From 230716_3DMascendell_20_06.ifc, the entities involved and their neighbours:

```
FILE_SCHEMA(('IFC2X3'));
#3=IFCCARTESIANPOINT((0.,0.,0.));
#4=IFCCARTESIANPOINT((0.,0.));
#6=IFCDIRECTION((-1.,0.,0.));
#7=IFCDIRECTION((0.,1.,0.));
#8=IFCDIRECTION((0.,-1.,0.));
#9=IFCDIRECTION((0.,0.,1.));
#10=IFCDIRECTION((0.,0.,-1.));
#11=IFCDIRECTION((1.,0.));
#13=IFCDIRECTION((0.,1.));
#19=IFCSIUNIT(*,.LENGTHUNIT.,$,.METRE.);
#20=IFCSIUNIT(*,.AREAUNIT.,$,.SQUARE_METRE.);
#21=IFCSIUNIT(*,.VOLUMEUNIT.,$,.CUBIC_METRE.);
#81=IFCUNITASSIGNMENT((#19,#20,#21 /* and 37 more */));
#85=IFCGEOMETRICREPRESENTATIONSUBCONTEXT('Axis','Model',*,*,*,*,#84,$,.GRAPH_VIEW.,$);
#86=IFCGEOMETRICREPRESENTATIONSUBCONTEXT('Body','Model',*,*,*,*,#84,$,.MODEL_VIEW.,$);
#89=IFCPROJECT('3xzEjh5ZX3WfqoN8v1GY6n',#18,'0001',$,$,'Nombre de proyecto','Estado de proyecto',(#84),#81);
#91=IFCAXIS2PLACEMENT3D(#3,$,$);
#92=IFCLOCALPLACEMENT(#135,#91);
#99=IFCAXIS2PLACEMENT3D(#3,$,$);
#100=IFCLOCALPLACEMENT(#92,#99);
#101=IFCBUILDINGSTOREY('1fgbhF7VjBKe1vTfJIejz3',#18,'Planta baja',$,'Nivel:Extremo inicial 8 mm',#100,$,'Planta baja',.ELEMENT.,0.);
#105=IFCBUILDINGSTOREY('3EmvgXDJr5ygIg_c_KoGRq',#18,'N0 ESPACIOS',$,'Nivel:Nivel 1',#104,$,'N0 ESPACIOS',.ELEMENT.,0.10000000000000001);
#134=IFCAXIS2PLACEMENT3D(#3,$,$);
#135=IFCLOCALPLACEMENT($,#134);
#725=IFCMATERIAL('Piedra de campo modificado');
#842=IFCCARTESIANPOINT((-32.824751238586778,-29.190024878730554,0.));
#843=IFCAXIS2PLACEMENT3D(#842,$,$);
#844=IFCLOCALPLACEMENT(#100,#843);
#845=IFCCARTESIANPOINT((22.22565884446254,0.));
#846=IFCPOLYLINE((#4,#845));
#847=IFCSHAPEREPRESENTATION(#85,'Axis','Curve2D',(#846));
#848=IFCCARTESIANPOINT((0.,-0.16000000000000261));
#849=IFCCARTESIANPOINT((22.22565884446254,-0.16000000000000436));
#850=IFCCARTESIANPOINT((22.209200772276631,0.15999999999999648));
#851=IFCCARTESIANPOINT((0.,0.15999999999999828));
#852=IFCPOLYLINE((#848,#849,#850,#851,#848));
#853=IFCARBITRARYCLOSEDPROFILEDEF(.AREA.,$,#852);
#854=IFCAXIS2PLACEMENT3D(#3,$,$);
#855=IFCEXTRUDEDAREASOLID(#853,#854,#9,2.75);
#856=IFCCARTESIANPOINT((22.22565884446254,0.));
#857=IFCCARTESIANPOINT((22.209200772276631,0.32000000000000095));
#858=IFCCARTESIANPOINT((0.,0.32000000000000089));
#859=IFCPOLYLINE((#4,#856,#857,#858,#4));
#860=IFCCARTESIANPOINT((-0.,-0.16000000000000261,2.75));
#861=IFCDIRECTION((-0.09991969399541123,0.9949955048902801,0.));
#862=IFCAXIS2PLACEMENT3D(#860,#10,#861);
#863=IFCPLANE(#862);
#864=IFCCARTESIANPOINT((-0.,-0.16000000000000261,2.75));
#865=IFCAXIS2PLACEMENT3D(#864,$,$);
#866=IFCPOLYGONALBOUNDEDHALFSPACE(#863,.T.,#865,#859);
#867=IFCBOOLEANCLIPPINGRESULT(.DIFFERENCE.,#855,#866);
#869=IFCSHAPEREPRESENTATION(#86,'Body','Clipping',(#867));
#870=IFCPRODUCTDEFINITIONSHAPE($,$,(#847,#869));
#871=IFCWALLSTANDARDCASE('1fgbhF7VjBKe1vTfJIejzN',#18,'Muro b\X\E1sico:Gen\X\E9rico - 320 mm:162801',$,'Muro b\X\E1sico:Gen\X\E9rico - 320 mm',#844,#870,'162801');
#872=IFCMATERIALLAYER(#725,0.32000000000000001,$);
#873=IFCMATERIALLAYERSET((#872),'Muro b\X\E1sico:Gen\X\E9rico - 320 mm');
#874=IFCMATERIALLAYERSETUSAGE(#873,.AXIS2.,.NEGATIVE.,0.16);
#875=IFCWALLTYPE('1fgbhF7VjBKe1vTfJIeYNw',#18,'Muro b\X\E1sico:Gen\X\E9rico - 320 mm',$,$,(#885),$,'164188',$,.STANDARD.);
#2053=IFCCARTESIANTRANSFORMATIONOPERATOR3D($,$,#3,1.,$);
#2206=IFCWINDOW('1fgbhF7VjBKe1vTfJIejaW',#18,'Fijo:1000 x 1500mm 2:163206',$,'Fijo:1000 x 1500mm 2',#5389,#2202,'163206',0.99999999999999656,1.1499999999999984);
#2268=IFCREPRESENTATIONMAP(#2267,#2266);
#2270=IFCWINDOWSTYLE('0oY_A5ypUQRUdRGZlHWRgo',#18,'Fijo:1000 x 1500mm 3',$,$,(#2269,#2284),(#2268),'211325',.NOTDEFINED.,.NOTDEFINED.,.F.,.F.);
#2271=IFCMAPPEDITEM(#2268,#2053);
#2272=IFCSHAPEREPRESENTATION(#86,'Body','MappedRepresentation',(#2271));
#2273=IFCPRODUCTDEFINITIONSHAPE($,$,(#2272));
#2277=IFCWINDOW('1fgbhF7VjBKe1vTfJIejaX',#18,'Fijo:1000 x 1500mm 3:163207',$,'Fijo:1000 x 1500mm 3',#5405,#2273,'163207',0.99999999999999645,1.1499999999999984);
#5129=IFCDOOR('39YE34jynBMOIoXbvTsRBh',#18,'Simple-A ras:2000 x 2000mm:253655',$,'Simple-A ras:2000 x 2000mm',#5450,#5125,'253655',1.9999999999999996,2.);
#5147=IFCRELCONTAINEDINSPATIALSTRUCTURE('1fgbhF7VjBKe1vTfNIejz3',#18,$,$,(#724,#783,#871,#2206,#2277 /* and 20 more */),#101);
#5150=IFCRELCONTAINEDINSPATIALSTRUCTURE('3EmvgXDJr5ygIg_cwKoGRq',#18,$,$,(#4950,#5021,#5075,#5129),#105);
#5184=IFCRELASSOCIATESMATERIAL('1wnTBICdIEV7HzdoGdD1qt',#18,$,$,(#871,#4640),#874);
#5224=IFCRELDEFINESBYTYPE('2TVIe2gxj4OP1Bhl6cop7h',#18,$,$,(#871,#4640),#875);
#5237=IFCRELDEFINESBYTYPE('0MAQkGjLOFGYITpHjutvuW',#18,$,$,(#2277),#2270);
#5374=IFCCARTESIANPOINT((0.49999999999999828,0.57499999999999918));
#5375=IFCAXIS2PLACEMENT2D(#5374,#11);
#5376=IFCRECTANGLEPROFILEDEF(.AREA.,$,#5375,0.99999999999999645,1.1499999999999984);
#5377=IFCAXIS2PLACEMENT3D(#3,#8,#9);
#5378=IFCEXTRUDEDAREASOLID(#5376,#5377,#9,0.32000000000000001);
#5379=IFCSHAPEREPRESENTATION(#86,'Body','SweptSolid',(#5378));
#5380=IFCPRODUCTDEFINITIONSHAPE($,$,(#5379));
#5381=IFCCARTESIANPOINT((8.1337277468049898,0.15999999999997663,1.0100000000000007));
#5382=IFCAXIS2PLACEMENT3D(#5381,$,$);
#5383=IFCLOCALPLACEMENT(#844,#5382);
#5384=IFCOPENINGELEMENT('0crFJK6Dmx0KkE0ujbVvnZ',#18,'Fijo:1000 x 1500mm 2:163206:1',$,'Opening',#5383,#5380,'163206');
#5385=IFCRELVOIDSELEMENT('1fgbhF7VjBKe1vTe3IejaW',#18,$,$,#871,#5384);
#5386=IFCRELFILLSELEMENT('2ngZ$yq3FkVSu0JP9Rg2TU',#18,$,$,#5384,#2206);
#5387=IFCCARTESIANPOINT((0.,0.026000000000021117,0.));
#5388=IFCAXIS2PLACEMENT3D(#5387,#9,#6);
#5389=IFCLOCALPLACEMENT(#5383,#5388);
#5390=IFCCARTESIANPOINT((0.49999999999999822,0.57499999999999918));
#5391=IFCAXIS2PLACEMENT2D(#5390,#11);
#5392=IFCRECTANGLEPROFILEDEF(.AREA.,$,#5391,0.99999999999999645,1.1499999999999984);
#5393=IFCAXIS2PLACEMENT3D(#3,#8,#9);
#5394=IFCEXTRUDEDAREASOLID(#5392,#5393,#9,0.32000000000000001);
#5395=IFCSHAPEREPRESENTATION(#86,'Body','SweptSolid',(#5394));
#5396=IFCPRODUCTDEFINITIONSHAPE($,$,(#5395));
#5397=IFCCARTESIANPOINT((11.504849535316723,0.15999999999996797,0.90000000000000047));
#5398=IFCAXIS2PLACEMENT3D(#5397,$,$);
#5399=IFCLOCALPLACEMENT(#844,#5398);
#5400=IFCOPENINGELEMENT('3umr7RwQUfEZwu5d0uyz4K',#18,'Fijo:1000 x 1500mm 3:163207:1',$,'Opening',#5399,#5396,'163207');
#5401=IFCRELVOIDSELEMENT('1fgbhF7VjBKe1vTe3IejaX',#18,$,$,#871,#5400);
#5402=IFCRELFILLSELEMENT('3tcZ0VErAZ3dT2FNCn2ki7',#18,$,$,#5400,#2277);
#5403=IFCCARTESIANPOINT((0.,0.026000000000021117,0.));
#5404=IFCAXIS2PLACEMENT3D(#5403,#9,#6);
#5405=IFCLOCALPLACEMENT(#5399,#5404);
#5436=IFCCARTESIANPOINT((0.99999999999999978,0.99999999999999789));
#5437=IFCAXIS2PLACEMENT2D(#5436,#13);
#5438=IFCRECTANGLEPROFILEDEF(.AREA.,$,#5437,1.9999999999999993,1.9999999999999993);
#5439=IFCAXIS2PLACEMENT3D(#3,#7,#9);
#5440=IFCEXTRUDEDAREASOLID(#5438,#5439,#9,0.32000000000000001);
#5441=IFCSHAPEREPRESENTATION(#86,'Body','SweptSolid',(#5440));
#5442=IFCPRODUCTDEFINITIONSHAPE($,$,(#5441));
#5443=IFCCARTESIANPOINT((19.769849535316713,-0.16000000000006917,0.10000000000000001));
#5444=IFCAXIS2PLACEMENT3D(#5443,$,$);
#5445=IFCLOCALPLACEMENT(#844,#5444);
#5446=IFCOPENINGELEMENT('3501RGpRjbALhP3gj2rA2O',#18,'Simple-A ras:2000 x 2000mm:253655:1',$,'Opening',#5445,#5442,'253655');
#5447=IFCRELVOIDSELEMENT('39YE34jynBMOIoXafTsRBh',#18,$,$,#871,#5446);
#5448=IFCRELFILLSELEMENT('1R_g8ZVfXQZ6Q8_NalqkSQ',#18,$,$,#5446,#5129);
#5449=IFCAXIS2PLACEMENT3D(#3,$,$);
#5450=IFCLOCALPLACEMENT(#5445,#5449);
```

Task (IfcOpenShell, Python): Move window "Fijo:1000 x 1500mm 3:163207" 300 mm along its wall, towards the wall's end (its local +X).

```python
import ifcopenshell
import ifcopenshell.api.geometry
import ifcopenshell.util.placement
import ifcopenshell.util.unit

model = ifcopenshell.open("230716_3DMascendell_20_06.ifc")
unit_scale = ifcopenshell.util.unit.calculate_unit_scale(model)

window = model.by_guid("1fgbhF7VjBKe1vTfJIejaX")
opening = window.FillsVoids[0].RelatingOpeningElement
wall = opening.VoidsElements[0].RelatingBuildingElement

wall_matrix = ifcopenshell.util.placement.get_local_placement(wall.ObjectPlacement)
shift = wall_matrix[:3, 0] * 0.3 / unit_scale
before = ifcopenshell.util.placement.get_local_placement(window.ObjectPlacement)[:3, 3].copy()

# The window is placed relative to its opening, so it follows when the opening moves.
matrix = ifcopenshell.util.placement.get_local_placement(opening.ObjectPlacement)
matrix[:3, 3] += shift
ifcopenshell.api.geometry.edit_object_placement(
    model, product=opening, matrix=matrix, is_si=False, should_transform_children=True
)

after = ifcopenshell.util.placement.get_local_placement(window.ObjectPlacement)[:3, 3]
print("window moved by", (after - before).round(3) + 0.0)

model.write("230716_3DMascendell_20_06_updated.ifc")
```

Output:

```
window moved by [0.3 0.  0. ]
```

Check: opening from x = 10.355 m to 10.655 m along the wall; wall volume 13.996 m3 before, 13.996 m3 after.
